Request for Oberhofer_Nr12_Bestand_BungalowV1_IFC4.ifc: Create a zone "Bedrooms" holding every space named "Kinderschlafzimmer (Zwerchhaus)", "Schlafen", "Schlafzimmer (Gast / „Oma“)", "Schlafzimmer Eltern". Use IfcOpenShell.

First a look at what the model holds.

```python
import ifcopenshell

model = ifcopenshell.open("Oberhofer_Nr12_Bestand_BungalowV1_IFC4.ifc")
print(model.schema)
seen = {}
for space in model.by_type("IfcSpace"):
    seen[space.LongName] = seen.get(space.LongName, 0) + 1
for name, count in sorted(seen.items(), key=str):
    print(count, "x", name)
print("zones:", [z.Name for z in model.by_type("IfcZone")][:20])
```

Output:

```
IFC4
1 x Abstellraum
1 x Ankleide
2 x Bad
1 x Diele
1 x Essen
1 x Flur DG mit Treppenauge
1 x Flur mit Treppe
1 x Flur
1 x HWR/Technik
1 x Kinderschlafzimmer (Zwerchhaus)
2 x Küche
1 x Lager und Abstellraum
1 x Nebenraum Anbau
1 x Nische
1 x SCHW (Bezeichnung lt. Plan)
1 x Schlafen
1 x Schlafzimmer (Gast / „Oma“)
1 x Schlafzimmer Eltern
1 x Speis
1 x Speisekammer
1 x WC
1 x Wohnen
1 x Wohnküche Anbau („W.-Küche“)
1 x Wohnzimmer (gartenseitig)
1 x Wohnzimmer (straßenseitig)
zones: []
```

```python
import ifcopenshell
import ifcopenshell.api.group
import ifcopenshell.api.root

model = ifcopenshell.open("Oberhofer_Nr12_Bestand_BungalowV1_IFC4.ifc")

names = {"Kinderschlafzimmer (Zwerchhaus)", "Schlafen", "Schlafzimmer (Gast / „Oma“)", "Schlafzimmer Eltern"}
spaces = [s for s in model.by_type("IfcSpace") if s.LongName in names]

zone = ifcopenshell.api.root.create_entity(model, ifc_class="IfcZone", name="Bedrooms")
ifcopenshell.api.group.assign_group(model, products=spaces, group=zone)
print(len(spaces), "spaces in", zone.Name)

model.write("Oberhofer_Nr12_Bestand_BungalowV1_IFC4_v2.ifc")
```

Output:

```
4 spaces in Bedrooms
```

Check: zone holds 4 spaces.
